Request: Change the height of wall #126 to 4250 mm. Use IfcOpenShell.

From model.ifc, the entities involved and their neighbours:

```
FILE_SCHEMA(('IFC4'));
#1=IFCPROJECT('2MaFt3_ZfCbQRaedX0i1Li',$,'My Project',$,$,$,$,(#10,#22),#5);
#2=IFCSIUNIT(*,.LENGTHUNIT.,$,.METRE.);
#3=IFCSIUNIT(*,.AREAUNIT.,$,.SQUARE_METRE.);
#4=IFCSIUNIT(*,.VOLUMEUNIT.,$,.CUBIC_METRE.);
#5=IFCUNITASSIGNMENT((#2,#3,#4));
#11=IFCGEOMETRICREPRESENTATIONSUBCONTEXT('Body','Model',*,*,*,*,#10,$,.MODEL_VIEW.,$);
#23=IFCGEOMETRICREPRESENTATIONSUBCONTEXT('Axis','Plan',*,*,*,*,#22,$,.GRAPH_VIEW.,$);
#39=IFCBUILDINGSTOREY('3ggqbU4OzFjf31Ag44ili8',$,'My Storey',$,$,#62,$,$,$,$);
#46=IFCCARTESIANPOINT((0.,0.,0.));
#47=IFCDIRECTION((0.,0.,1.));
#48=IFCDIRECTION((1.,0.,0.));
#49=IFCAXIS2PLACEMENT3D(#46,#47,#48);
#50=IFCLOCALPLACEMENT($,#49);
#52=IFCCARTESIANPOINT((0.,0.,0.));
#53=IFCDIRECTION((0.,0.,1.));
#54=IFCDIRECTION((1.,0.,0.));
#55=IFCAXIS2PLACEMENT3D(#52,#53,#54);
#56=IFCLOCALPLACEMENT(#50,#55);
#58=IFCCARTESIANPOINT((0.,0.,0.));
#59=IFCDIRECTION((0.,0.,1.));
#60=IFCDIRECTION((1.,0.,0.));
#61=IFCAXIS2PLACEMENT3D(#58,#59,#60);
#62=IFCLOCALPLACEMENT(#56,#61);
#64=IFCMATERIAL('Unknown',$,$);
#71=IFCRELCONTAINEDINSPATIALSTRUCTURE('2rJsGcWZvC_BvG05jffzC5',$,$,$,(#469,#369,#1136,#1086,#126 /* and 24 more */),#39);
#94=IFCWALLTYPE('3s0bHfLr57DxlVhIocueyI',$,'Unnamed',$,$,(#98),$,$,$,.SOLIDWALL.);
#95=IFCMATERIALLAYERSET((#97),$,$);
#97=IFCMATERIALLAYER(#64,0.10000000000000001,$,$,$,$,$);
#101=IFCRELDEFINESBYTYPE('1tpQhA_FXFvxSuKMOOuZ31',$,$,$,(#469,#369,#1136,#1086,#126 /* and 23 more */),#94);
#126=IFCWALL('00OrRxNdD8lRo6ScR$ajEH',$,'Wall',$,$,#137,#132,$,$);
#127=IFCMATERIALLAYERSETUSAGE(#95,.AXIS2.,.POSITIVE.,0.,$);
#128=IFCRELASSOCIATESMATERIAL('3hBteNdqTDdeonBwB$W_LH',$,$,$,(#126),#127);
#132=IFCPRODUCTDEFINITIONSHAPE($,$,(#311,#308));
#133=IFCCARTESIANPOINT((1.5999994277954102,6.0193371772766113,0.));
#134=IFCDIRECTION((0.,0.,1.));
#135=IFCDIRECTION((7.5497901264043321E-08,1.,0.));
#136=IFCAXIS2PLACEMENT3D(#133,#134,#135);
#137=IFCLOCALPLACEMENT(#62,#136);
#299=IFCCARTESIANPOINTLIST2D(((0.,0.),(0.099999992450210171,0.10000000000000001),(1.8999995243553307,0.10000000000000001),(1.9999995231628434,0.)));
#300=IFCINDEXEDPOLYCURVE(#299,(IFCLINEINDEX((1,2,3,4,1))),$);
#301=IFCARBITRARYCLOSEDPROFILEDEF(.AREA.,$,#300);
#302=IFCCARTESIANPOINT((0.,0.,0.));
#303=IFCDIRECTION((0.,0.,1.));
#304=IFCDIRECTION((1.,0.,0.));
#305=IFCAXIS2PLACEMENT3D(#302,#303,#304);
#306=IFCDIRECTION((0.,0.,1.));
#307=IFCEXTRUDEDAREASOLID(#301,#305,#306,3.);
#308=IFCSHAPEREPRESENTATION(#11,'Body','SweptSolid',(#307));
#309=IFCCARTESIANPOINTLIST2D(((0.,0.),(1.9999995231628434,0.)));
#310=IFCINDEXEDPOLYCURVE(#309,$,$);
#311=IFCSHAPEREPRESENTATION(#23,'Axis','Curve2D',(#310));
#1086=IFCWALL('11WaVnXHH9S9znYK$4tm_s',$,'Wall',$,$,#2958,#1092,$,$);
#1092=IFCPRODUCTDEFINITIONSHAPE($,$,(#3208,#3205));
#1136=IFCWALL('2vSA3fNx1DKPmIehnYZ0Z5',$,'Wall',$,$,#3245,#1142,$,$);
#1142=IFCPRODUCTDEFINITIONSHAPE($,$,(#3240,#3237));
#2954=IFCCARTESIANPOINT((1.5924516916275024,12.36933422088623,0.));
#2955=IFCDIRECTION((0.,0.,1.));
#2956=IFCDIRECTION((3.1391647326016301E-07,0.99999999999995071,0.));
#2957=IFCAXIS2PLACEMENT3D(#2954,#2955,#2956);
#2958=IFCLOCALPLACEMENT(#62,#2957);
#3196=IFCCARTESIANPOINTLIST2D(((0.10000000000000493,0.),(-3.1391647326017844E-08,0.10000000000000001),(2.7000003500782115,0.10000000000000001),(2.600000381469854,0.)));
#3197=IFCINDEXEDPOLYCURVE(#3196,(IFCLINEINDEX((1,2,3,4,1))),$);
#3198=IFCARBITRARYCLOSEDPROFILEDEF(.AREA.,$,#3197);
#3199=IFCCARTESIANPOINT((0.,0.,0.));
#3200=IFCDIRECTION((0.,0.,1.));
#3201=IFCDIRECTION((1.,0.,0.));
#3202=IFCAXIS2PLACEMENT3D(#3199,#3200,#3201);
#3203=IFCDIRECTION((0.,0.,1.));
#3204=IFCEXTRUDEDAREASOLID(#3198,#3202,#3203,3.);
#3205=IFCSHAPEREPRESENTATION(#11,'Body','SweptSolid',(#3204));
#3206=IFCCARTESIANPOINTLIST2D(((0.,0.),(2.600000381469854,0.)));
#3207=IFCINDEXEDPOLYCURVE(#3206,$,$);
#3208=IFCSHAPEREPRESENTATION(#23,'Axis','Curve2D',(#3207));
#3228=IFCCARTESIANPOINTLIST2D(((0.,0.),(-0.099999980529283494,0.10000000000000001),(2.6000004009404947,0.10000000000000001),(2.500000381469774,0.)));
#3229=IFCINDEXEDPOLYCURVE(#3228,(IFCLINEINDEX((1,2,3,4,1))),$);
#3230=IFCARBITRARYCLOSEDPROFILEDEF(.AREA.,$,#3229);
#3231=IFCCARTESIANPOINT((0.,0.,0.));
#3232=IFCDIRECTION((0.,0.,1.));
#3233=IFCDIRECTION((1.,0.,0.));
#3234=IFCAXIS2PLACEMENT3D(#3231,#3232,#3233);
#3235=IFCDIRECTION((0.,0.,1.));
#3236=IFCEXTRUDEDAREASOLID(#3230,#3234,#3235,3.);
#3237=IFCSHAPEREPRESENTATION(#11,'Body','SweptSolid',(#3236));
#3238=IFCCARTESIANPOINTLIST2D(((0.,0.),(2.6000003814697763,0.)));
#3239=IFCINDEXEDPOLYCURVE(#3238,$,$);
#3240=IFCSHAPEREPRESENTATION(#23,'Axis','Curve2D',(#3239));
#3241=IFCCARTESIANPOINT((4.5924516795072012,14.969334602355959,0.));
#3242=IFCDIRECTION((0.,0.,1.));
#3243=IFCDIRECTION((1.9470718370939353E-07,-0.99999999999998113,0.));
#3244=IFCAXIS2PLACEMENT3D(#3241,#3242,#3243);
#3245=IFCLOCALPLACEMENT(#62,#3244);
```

```python
import ifcopenshell
import ifcopenshell.geom
import ifcopenshell.util.representation
import ifcopenshell.util.shape
import ifcopenshell.util.unit

model = ifcopenshell.open("model.ifc")
unit_scale = ifcopenshell.util.unit.calculate_unit_scale(model)
settings = ifcopenshell.geom.settings()


def volume(element):
    """Net volume in cubic metres, openings subtracted."""
    shape = ifcopenshell.geom.create_shape(settings, element)
    return ifcopenshell.util.shape.get_volume(shape.geometry)


wall = model.by_guid("00OrRxNdD8lRo6ScR$ajEH")
before = volume(wall)

body = ifcopenshell.util.representation.get_representation(wall, "Model", "Body")
solid = body.Items[0]
old_height = solid.Depth
solid.Depth = 4.25 / unit_scale
after = volume(wall)

print(f"height {old_height:g} -> {solid.Depth:g}, volume {before:.3f} -> {after:.3f} m3")

model.write("model_updated.ifc")
```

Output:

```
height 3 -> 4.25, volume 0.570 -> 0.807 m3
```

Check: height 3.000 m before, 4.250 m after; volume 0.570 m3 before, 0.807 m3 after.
